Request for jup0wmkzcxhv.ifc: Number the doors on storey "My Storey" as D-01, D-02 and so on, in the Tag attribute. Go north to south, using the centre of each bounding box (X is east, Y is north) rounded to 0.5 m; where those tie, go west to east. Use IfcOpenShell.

First a look at what the model holds.

```python
import ifcopenshell
import ifcopenshell.util.element
import ifcopenshell.util.placement

model = ifcopenshell.open("jup0wmkzcxhv.ifc")
print(model.schema)
storey = next(s for s in model.by_type("IfcBuildingStorey") if s.Name == "My Storey")
doors = [e for e in ifcopenshell.util.element.get_decomposition(storey) if e.is_a("IfcDoor")]
for e in sorted(doors, key=lambda e: e.id()):
    origin = ifcopenshell.util.placement.get_local_placement(e.ObjectPlacement)[:3, 3]
    print(e.id(), e.Tag, e.Name, origin.round(2) + 0.0, sep=" | ")
```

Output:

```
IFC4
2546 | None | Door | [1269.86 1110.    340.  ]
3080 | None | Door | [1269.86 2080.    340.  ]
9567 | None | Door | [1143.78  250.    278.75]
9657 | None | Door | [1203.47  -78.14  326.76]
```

```python
import ifcopenshell
import ifcopenshell.geom
import ifcopenshell.util.element
import ifcopenshell.util.shape

model = ifcopenshell.open("jup0wmkzcxhv.ifc")
settings = ifcopenshell.geom.settings()
settings.set("use-world-coords", True)


def centre(element):
    shape = ifcopenshell.geom.create_shape(settings, element)
    return ifcopenshell.util.shape.get_bbox_centroid(shape.geometry)


storey = next(s for s in model.by_type("IfcBuildingStorey") if s.Name == "My Storey")
doors = [e for e in ifcopenshell.util.element.get_decomposition(storey) if e.is_a("IfcDoor")]

# Insertion points can sit at a corner or the storey origin, so sort by the geometry (in metres).
centres = {e: centre(e) for e in doors}
doors.sort(key=lambda e: (-round(centres[e][1] / 0.5), centres[e][0]))

for i, e in enumerate(doors, start=1):
    number = f"D-{i:02d}"
    e.Tag = number
    print(e.id(), number)

model.write("jup0wmkzcxhv_updated.ifc")
```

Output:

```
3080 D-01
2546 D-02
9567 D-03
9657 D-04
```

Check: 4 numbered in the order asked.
